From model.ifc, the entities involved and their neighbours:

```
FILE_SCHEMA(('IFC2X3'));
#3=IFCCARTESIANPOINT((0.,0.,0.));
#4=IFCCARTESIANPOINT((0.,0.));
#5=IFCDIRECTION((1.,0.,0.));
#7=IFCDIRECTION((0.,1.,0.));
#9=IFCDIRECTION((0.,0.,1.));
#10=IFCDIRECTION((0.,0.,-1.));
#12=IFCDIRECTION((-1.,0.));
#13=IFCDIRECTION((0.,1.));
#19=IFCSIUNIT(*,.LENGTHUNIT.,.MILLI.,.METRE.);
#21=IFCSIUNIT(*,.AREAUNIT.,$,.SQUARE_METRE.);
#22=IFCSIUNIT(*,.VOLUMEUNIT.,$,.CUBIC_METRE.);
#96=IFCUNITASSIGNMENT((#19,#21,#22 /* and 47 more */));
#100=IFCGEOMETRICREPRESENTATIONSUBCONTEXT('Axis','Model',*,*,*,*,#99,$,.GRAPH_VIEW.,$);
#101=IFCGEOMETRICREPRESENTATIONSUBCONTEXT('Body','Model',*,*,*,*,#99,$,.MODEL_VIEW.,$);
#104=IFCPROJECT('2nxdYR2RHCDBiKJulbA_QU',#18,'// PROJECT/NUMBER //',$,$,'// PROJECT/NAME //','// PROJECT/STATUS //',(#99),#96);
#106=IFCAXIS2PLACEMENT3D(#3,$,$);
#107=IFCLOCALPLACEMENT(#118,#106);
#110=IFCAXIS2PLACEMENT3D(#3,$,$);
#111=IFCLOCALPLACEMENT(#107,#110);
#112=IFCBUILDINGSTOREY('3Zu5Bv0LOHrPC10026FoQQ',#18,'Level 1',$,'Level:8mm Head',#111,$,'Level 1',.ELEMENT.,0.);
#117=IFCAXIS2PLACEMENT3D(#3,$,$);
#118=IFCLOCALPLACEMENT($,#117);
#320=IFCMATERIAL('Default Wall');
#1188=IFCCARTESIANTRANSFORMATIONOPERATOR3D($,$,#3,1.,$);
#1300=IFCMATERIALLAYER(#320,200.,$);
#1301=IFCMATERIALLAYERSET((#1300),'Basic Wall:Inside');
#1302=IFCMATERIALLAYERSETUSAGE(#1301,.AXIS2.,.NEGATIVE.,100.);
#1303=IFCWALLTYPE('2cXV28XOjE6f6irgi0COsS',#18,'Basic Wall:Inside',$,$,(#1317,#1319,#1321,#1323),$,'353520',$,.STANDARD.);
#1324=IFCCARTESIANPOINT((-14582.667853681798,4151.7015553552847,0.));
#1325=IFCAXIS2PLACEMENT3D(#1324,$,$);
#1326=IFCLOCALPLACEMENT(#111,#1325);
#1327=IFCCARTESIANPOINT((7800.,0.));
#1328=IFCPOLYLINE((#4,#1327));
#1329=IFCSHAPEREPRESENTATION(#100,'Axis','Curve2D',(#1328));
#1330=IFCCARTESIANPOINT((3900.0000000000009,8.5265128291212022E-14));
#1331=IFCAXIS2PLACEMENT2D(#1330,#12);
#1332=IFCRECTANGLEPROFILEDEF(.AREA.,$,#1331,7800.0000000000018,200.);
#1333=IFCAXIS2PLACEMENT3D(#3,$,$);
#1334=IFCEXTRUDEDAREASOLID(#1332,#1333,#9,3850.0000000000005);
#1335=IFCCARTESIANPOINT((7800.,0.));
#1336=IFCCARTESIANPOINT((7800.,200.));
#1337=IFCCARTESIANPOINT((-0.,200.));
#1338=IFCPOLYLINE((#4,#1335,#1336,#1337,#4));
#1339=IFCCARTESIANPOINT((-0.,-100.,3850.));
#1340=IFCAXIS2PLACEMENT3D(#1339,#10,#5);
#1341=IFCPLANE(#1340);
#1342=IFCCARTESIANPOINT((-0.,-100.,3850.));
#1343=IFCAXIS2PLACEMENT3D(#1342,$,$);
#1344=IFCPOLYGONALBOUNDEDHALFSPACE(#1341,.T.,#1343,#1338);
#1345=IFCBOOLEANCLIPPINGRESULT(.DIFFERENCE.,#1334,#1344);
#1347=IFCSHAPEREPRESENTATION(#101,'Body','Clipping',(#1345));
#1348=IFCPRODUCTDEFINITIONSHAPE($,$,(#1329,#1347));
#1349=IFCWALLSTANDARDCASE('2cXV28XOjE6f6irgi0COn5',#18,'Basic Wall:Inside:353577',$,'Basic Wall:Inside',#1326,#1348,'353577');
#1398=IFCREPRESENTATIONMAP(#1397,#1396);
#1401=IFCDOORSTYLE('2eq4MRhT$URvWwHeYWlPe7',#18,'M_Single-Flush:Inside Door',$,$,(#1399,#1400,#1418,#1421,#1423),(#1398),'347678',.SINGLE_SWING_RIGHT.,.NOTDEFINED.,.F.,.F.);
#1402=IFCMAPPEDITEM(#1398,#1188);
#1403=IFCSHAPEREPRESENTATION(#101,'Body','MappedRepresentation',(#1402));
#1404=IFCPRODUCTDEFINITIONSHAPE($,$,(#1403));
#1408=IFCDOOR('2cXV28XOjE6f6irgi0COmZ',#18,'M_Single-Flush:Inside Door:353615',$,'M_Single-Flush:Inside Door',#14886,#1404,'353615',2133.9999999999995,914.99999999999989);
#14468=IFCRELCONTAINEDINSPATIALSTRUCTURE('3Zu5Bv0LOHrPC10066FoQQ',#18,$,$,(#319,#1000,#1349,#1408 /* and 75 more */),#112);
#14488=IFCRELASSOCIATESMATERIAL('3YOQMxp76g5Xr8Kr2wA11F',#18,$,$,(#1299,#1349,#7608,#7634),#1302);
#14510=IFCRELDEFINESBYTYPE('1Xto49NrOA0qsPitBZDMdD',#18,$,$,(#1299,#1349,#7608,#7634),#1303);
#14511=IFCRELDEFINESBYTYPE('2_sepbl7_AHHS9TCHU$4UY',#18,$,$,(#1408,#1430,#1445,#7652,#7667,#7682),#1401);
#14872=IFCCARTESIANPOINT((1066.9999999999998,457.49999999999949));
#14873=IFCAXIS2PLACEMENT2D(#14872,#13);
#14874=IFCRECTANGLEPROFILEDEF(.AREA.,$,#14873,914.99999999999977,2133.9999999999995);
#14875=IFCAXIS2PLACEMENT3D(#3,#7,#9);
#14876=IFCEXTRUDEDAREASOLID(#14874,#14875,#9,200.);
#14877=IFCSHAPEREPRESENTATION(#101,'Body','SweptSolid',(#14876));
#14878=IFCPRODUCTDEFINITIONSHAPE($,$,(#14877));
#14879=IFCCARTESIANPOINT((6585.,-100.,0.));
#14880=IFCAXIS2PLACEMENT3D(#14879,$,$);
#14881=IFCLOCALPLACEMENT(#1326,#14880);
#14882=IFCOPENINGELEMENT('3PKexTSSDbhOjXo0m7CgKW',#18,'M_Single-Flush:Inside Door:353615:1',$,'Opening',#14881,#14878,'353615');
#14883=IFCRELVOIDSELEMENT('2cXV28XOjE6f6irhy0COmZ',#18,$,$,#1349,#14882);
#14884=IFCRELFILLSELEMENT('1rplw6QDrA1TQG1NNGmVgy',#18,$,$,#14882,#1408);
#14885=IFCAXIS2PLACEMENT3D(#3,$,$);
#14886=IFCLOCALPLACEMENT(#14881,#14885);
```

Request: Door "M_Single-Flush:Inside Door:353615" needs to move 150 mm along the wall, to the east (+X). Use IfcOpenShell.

```python
import ifcopenshell
import ifcopenshell.api.geometry
import ifcopenshell.util.placement

model = ifcopenshell.open("model.ifc")

door = model.by_guid("2cXV28XOjE6f6irgi0COmZ")
opening = door.FillsVoids[0].RelatingOpeningElement
wall = opening.VoidsElements[0].RelatingBuildingElement

wall_matrix = ifcopenshell.util.placement.get_local_placement(wall.ObjectPlacement)
shift = wall_matrix[:3, 0] * 150.0
before = ifcopenshell.util.placement.get_local_placement(door.ObjectPlacement)[:3, 3].copy()

# The door is placed relative to its opening, so it follows when the opening moves.
matrix = ifcopenshell.util.placement.get_local_placement(opening.ObjectPlacement)
matrix[:3, 3] += shift
ifcopenshell.api.geometry.edit_object_placement(
    model, product=opening, matrix=matrix, is_si=False, should_transform_children=True
)

after = ifcopenshell.util.placement.get_local_placement(door.ObjectPlacement)[:3, 3]
print("door moved by", (after - before).round(3) + 0.0)

model.write("model_v2.ifc")
```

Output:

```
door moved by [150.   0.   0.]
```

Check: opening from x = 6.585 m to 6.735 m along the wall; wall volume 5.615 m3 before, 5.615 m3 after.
